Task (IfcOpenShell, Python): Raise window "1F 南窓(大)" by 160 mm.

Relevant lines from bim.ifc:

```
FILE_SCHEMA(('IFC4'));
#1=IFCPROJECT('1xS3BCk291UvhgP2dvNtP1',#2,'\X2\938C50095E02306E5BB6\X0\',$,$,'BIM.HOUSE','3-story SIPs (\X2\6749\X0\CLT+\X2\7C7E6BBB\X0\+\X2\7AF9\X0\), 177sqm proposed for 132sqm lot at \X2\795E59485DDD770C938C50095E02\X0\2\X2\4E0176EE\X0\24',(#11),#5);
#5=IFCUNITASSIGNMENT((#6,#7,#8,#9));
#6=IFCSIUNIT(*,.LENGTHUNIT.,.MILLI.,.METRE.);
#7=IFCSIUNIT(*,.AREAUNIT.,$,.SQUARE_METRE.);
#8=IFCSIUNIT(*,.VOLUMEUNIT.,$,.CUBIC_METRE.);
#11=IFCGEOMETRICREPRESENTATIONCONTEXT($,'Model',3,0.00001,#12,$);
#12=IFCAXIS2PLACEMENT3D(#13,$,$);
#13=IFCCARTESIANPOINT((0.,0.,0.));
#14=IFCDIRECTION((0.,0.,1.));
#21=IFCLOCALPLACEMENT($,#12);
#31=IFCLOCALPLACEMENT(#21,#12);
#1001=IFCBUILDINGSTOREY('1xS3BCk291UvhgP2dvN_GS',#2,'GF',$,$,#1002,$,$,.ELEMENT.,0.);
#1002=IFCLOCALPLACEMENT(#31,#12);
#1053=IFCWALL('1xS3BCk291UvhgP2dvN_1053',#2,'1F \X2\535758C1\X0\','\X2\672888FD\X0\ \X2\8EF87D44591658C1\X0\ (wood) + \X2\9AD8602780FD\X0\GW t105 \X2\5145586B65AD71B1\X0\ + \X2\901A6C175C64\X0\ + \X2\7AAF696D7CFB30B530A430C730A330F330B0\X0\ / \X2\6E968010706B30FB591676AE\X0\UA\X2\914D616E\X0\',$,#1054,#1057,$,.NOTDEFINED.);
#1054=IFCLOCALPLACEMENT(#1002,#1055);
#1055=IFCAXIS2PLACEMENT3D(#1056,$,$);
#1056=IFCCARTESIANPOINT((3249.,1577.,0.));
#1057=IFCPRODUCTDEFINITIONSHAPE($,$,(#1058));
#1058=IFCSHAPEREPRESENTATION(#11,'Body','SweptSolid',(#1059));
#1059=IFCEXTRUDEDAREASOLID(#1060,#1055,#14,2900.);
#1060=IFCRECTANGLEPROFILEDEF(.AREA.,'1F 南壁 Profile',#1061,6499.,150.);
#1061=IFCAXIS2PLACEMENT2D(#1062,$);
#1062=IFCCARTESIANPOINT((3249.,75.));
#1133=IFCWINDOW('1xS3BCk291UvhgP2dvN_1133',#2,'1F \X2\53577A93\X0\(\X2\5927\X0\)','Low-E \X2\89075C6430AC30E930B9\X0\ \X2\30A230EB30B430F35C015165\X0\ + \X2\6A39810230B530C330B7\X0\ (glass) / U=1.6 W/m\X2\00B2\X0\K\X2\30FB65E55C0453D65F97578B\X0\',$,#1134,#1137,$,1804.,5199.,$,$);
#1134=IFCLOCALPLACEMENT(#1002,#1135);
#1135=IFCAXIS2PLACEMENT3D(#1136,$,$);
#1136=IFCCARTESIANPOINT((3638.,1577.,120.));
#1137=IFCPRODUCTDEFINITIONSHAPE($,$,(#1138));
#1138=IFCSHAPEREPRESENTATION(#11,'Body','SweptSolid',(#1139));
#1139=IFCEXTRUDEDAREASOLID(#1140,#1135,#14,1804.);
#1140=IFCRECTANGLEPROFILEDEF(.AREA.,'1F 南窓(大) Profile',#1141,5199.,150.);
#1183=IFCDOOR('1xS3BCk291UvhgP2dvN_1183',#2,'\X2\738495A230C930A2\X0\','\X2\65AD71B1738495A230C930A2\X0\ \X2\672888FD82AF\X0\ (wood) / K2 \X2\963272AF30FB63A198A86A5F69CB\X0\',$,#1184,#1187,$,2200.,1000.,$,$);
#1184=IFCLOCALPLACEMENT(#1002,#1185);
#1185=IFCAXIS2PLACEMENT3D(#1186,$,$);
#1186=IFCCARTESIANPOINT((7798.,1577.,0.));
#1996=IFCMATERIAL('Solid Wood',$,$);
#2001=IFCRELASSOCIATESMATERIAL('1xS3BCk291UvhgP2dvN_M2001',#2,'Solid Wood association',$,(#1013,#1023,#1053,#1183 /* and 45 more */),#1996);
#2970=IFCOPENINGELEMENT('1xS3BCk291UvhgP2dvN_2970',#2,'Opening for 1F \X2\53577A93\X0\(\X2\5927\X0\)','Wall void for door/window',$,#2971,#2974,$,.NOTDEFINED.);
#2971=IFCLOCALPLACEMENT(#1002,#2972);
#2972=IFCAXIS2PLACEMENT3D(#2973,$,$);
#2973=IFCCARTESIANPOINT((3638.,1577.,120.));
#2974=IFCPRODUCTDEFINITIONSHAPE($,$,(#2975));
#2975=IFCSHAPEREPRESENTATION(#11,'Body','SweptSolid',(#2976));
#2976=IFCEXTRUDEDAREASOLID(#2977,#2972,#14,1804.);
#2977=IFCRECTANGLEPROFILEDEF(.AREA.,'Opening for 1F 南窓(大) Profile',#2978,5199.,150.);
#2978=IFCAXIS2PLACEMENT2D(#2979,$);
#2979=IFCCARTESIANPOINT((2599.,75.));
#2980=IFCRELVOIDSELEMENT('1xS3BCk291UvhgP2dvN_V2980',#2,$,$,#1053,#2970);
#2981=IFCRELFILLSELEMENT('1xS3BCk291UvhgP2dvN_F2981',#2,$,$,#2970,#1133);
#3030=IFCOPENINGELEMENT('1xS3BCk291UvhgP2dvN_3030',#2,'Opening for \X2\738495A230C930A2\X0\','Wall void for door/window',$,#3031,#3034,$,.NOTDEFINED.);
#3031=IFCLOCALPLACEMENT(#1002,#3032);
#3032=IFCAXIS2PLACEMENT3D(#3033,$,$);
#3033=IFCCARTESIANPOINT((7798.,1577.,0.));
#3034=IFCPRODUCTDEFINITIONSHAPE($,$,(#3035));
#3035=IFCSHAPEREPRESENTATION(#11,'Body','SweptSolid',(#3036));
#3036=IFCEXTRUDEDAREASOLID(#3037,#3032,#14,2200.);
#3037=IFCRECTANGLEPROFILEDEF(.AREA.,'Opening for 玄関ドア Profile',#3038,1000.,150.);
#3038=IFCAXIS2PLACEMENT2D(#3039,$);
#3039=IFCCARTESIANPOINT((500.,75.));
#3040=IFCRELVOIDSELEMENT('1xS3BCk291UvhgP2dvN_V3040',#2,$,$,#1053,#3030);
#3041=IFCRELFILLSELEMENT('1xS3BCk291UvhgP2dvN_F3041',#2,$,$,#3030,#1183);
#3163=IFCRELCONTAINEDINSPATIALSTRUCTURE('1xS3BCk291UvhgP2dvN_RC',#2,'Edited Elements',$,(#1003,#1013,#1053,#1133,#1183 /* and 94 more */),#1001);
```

```python
import numpy as np
import ifcopenshell
import ifcopenshell.api.geometry
import ifcopenshell.util.placement
import ifcopenshell.util.unit

model = ifcopenshell.open("bim.ifc")
unit_scale = ifcopenshell.util.unit.calculate_unit_scale(model)

window = model.by_guid("1xS3BCk291UvhgP2dvN_1133")
opening = window.FillsVoids[0].RelatingOpeningElement
dz = 160.0

shift = np.array([0.0, 0.0, dz])
# The window is not placed relative to its opening, so move both.
for product in (opening, window):
    matrix = ifcopenshell.util.placement.get_local_placement(product.ObjectPlacement)
    matrix[:3, 3] += shift
    ifcopenshell.api.geometry.edit_object_placement(model, product=product, matrix=matrix, is_si=False)

print(f"moved by {dz * unit_scale:+.3f} m")

model.write("bim_v2.ifc")
```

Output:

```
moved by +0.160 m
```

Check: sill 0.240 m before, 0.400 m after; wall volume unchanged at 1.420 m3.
